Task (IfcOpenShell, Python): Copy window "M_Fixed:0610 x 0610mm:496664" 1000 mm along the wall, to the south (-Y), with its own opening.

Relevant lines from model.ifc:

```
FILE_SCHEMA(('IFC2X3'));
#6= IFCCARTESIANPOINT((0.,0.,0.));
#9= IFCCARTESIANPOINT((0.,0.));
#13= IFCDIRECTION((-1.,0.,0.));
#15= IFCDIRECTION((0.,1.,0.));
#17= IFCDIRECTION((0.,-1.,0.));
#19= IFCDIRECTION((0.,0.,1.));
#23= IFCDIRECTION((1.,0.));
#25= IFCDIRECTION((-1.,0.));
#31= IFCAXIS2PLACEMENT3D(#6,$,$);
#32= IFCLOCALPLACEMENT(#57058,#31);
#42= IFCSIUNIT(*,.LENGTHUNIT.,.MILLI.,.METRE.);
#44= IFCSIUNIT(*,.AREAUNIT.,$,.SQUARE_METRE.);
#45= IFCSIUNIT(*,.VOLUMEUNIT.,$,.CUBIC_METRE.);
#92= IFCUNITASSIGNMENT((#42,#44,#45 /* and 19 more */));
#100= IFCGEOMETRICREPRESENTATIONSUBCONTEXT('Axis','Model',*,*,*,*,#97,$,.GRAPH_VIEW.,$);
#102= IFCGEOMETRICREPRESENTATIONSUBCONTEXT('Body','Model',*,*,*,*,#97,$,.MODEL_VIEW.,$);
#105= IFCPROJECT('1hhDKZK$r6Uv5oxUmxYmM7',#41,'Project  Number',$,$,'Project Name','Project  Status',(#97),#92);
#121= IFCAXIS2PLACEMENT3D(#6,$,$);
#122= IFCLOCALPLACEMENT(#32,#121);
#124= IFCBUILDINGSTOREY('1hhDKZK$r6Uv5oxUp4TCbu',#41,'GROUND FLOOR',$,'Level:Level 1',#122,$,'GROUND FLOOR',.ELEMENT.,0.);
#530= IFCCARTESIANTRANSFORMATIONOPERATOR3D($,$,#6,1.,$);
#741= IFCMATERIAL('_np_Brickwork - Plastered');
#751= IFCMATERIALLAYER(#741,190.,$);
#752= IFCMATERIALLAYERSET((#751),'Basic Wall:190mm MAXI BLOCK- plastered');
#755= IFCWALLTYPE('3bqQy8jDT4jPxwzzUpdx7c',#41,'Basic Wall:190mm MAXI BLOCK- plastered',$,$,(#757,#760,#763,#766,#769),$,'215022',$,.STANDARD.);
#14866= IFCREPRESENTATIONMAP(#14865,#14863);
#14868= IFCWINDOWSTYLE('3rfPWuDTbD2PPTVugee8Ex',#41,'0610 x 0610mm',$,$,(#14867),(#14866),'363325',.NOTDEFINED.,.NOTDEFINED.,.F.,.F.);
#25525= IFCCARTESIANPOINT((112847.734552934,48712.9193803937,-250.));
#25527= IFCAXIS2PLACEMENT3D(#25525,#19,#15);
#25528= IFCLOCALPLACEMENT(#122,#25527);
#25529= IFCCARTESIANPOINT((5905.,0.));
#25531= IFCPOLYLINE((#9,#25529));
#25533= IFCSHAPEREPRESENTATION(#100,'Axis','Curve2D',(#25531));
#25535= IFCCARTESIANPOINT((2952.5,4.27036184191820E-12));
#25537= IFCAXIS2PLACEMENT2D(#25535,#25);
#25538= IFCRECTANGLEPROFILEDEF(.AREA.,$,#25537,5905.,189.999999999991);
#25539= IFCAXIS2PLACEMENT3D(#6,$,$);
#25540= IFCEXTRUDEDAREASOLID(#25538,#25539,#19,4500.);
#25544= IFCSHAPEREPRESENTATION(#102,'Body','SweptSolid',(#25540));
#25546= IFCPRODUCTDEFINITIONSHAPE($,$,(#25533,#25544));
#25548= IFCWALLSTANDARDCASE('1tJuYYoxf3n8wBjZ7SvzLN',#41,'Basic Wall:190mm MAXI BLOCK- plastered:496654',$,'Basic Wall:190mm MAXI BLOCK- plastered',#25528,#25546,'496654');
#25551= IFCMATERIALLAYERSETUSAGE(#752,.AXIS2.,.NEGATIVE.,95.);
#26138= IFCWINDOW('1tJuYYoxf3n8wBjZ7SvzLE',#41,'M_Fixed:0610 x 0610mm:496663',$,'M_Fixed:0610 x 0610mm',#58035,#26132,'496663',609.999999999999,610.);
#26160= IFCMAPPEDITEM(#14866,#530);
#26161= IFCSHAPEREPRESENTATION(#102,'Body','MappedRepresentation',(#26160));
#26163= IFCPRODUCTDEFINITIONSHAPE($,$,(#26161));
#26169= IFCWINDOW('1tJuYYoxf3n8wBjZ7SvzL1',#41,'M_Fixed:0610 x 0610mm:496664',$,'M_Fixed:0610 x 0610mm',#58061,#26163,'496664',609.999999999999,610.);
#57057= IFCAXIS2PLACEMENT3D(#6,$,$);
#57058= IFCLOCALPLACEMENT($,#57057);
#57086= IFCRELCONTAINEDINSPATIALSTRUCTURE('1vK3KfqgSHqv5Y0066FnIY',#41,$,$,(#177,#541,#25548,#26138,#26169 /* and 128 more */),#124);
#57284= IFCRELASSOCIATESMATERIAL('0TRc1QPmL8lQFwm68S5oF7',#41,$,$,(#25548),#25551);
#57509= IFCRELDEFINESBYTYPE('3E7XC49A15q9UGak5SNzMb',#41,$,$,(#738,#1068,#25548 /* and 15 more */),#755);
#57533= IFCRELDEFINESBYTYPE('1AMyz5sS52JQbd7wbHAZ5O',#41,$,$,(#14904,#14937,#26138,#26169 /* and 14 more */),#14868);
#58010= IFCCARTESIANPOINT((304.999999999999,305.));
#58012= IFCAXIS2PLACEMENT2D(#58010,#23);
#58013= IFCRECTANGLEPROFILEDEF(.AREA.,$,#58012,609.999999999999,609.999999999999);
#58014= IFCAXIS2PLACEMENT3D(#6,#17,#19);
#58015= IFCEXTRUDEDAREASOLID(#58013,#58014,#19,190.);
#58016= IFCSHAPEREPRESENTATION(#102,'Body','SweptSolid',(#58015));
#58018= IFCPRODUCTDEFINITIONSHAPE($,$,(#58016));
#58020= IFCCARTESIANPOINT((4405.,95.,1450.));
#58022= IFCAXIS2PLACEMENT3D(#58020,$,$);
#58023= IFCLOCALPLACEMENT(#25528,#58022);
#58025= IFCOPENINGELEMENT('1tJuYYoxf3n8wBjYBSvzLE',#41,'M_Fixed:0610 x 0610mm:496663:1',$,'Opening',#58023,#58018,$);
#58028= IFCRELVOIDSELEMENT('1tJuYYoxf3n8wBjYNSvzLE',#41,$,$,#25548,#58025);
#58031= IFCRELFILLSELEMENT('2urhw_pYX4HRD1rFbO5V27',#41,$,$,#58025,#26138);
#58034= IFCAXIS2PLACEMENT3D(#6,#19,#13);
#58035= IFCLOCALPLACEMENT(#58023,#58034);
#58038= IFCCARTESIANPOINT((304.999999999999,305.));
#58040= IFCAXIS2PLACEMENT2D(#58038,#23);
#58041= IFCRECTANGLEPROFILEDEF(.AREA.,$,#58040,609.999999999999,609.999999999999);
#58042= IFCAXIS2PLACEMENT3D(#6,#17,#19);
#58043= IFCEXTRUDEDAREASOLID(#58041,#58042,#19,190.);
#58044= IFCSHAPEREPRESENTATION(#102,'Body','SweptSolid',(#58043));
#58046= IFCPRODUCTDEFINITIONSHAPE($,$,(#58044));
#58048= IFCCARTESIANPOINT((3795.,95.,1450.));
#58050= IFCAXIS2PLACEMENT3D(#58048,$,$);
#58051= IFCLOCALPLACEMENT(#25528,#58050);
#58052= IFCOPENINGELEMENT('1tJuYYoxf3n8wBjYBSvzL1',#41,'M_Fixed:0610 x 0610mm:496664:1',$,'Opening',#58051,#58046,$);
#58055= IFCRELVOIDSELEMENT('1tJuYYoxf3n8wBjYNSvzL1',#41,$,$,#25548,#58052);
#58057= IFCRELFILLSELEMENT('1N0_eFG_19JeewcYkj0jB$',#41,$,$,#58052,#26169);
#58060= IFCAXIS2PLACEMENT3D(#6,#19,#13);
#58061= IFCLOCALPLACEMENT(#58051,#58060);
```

```python
import ifcopenshell
import ifcopenshell.api.feature
import ifcopenshell.api.geometry
import ifcopenshell.api.root
import ifcopenshell.geom
import ifcopenshell.util.element
import ifcopenshell.util.placement
import ifcopenshell.util.shape
import ifcopenshell.util.unit

model = ifcopenshell.open("model.ifc")
unit_scale = ifcopenshell.util.unit.calculate_unit_scale(model)
settings = ifcopenshell.geom.settings()


def volume(element):
    """Net volume in cubic metres, openings subtracted."""
    shape = ifcopenshell.geom.create_shape(settings, element)
    return ifcopenshell.util.shape.get_volume(shape.geometry)


def reuse_history(source, copy):
    """copy_class also copies each property set's owner history, people and application; keep the originals."""
    for rel in copy.IsDefinedBy:
        if rel.is_a("IfcRelDefinesByProperties") and (history := rel.RelatingPropertyDefinition.OwnerHistory):
            rel.RelatingPropertyDefinition.OwnerHistory = source.OwnerHistory
            ifcopenshell.util.element.remove_deep2(model, history)


window = model.by_guid("1tJuYYoxf3n8wBjZ7SvzL1")
opening = window.FillsVoids[0].RelatingOpeningElement
wall = opening.VoidsElements[0].RelatingBuildingElement
before = volume(wall)
shift = ifcopenshell.util.placement.get_local_placement(wall.ObjectPlacement)[:3, 0] * -1 / unit_scale

# copy_class copies the void relationship, type, container and properties, but no geometry.
new_opening = ifcopenshell.api.root.copy_class(model, product=opening)
new_opening.Representation = ifcopenshell.util.element.copy_deep(
    model, opening.Representation, exclude=["IfcGeometricRepresentationContext", "IfcRepresentationMap"]
)
new_opening.Name = "M_Fixed:0610 x 0610mm"
new_window = ifcopenshell.api.root.copy_class(model, product=window)
new_window.Representation = ifcopenshell.util.element.copy_deep(
    model, window.Representation, exclude=["IfcGeometricRepresentationContext", "IfcRepresentationMap"]
)
new_window.Name = "M_Fixed:0610 x 0610mm"
new_window.Tag = None
reuse_history(window, new_window)
fills = ifcopenshell.api.feature.add_filling(model, opening=new_opening, element=new_window)
fills.OwnerHistory = new_window.OwnerHistory  # required in IFC2X3

for old, new in ((opening, new_opening), (window, new_window)):
    matrix = ifcopenshell.util.placement.get_local_placement(old.ObjectPlacement)
    matrix[:3, 3] += shift
    ifcopenshell.api.geometry.edit_object_placement(model, product=new, matrix=matrix, is_si=False)

after = volume(wall)

print(f"wall volume {before:.3f} -> {after:.3f} m3")

model.write("model_updated.ifc")
```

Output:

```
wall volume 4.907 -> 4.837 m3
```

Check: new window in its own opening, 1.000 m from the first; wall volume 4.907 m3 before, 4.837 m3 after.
